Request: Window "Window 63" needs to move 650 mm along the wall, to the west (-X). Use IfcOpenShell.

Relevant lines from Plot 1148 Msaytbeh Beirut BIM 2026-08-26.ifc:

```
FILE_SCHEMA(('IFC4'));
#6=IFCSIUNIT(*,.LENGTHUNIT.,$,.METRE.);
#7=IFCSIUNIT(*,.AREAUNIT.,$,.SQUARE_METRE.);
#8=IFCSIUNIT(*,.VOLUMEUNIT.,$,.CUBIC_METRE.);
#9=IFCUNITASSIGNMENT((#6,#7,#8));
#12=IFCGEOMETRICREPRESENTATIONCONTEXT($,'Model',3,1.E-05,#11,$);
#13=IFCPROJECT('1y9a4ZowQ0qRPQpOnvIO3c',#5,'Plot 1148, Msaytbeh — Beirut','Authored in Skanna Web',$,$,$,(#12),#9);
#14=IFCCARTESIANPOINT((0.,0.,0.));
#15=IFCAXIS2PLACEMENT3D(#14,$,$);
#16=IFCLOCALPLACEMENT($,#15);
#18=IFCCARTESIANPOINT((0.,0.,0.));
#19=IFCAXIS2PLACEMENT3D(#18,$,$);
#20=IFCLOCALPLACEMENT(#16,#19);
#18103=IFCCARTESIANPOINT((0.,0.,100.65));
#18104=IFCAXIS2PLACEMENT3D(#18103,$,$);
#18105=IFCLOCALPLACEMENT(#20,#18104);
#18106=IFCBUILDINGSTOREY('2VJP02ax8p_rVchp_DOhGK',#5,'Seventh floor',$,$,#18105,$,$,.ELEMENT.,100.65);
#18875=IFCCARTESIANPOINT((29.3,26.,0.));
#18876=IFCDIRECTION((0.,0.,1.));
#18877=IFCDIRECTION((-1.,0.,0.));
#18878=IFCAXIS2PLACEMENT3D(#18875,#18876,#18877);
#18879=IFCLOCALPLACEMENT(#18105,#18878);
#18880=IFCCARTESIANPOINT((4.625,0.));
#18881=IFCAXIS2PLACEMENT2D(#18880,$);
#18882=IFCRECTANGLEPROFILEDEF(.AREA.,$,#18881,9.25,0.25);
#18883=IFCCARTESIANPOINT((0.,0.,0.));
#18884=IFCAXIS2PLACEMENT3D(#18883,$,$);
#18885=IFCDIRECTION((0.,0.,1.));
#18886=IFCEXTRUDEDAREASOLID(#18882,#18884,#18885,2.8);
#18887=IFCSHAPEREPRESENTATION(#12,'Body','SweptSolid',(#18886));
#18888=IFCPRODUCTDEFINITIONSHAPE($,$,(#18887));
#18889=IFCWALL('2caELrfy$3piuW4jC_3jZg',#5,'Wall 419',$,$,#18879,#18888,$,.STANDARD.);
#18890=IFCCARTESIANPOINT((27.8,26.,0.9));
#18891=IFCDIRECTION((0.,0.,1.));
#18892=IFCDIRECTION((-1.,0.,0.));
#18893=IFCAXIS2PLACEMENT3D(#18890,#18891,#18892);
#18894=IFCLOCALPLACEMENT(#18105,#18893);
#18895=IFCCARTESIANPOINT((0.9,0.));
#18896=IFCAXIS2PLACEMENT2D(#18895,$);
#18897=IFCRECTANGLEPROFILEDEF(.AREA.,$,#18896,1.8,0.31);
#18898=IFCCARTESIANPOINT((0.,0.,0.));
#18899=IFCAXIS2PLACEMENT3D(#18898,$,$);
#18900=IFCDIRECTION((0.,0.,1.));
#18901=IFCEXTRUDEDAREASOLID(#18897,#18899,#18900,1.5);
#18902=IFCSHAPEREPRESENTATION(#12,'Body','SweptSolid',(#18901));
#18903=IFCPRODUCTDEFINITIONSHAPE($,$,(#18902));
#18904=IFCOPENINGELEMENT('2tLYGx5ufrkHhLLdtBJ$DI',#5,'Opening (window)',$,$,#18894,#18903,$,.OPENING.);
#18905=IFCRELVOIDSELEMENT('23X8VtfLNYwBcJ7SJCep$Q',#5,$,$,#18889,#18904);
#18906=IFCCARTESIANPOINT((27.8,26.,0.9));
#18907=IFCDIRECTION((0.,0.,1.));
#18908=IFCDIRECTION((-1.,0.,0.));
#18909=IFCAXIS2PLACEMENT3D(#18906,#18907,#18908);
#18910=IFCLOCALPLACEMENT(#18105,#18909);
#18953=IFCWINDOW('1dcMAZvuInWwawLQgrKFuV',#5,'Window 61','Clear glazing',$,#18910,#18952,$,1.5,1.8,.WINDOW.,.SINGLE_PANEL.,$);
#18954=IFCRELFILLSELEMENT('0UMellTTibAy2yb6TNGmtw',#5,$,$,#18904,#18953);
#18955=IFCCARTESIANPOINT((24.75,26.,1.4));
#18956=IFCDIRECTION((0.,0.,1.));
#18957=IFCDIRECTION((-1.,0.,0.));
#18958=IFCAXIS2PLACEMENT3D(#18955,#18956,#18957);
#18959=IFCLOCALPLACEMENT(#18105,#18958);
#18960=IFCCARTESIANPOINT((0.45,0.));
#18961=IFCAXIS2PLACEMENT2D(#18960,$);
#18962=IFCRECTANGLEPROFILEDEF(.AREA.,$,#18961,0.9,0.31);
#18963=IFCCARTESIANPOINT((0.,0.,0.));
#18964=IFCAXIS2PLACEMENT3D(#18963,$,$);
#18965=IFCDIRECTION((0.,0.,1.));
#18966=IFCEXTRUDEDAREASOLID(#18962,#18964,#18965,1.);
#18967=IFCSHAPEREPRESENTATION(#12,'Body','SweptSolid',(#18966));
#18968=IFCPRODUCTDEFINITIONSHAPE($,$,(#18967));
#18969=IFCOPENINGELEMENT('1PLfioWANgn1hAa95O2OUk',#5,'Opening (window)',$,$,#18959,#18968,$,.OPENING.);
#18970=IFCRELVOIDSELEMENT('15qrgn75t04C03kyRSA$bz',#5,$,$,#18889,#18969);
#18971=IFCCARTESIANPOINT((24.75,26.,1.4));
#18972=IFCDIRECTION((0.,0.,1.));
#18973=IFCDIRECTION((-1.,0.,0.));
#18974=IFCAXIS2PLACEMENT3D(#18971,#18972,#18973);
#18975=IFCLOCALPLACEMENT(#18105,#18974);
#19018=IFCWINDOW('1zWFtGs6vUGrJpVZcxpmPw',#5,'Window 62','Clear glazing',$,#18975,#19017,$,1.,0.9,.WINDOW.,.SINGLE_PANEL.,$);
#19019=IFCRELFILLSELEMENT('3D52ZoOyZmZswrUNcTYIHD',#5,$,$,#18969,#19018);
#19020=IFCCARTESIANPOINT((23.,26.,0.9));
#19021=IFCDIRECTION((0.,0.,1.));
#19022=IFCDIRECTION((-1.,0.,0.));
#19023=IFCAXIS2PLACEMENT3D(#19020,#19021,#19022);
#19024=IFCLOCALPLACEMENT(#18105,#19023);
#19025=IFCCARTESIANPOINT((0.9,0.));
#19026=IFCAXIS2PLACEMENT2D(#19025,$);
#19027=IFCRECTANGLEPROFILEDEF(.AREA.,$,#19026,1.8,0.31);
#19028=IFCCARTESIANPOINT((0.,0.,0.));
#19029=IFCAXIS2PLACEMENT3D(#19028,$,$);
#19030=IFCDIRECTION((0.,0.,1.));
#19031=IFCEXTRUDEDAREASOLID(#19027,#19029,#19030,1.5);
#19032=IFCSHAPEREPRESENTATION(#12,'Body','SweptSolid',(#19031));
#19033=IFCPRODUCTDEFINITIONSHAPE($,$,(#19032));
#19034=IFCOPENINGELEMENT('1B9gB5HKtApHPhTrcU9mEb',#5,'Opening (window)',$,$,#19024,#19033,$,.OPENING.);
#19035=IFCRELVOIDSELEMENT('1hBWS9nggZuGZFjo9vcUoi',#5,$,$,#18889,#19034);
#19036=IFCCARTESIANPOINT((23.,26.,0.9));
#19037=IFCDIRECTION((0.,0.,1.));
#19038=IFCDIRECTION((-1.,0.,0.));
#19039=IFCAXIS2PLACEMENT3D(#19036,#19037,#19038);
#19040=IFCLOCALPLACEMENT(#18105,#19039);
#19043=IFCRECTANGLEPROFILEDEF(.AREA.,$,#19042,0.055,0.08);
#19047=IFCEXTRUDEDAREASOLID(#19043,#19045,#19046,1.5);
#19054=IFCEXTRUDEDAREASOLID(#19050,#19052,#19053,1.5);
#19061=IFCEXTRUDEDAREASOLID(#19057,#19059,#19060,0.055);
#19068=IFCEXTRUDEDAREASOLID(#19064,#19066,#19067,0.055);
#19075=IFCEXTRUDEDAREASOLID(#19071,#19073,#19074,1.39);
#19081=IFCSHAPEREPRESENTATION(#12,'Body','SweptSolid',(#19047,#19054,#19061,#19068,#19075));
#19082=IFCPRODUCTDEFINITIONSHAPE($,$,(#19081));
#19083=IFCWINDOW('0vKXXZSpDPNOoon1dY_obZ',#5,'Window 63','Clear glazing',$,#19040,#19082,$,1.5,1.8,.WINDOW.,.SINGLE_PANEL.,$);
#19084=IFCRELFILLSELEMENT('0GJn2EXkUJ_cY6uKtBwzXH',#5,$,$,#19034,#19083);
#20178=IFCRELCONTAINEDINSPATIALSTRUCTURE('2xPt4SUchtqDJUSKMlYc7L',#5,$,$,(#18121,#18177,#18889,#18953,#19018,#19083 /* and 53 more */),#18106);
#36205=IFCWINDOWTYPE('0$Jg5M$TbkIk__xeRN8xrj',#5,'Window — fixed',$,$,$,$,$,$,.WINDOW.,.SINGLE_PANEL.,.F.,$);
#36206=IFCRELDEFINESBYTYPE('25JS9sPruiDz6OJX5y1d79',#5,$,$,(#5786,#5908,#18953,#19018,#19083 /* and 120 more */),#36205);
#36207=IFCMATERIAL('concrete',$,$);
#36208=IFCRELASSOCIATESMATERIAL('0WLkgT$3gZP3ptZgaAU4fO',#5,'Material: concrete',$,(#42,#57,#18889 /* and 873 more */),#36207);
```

```python
import ifcopenshell
import ifcopenshell.api.geometry
import ifcopenshell.util.placement

model = ifcopenshell.open("Plot 1148 Msaytbeh Beirut BIM 2026-08-26.ifc")

window = model.by_id(19083)
opening = window.FillsVoids[0].RelatingOpeningElement
wall = opening.VoidsElements[0].RelatingBuildingElement

wall_matrix = ifcopenshell.util.placement.get_local_placement(wall.ObjectPlacement)
shift = wall_matrix[:3, 0] * 0.65
before = ifcopenshell.util.placement.get_local_placement(window.ObjectPlacement)[:3, 3].copy()

# The window is not placed relative to its opening, so move both.
for product in (opening, window):
    matrix = ifcopenshell.util.placement.get_local_placement(product.ObjectPlacement)
    matrix[:3, 3] += shift
    ifcopenshell.api.geometry.edit_object_placement(model, product=product, matrix=matrix, is_si=False)

after = ifcopenshell.util.placement.get_local_placement(window.ObjectPlacement)[:3, 3]
print("window moved by", (after - before).round(3) + 0.0)

model.write("Plot 1148 Msaytbeh Beirut BIM 2026-08-26-out.ifc")
```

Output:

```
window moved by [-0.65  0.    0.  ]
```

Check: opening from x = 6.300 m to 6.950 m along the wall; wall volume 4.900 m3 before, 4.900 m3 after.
